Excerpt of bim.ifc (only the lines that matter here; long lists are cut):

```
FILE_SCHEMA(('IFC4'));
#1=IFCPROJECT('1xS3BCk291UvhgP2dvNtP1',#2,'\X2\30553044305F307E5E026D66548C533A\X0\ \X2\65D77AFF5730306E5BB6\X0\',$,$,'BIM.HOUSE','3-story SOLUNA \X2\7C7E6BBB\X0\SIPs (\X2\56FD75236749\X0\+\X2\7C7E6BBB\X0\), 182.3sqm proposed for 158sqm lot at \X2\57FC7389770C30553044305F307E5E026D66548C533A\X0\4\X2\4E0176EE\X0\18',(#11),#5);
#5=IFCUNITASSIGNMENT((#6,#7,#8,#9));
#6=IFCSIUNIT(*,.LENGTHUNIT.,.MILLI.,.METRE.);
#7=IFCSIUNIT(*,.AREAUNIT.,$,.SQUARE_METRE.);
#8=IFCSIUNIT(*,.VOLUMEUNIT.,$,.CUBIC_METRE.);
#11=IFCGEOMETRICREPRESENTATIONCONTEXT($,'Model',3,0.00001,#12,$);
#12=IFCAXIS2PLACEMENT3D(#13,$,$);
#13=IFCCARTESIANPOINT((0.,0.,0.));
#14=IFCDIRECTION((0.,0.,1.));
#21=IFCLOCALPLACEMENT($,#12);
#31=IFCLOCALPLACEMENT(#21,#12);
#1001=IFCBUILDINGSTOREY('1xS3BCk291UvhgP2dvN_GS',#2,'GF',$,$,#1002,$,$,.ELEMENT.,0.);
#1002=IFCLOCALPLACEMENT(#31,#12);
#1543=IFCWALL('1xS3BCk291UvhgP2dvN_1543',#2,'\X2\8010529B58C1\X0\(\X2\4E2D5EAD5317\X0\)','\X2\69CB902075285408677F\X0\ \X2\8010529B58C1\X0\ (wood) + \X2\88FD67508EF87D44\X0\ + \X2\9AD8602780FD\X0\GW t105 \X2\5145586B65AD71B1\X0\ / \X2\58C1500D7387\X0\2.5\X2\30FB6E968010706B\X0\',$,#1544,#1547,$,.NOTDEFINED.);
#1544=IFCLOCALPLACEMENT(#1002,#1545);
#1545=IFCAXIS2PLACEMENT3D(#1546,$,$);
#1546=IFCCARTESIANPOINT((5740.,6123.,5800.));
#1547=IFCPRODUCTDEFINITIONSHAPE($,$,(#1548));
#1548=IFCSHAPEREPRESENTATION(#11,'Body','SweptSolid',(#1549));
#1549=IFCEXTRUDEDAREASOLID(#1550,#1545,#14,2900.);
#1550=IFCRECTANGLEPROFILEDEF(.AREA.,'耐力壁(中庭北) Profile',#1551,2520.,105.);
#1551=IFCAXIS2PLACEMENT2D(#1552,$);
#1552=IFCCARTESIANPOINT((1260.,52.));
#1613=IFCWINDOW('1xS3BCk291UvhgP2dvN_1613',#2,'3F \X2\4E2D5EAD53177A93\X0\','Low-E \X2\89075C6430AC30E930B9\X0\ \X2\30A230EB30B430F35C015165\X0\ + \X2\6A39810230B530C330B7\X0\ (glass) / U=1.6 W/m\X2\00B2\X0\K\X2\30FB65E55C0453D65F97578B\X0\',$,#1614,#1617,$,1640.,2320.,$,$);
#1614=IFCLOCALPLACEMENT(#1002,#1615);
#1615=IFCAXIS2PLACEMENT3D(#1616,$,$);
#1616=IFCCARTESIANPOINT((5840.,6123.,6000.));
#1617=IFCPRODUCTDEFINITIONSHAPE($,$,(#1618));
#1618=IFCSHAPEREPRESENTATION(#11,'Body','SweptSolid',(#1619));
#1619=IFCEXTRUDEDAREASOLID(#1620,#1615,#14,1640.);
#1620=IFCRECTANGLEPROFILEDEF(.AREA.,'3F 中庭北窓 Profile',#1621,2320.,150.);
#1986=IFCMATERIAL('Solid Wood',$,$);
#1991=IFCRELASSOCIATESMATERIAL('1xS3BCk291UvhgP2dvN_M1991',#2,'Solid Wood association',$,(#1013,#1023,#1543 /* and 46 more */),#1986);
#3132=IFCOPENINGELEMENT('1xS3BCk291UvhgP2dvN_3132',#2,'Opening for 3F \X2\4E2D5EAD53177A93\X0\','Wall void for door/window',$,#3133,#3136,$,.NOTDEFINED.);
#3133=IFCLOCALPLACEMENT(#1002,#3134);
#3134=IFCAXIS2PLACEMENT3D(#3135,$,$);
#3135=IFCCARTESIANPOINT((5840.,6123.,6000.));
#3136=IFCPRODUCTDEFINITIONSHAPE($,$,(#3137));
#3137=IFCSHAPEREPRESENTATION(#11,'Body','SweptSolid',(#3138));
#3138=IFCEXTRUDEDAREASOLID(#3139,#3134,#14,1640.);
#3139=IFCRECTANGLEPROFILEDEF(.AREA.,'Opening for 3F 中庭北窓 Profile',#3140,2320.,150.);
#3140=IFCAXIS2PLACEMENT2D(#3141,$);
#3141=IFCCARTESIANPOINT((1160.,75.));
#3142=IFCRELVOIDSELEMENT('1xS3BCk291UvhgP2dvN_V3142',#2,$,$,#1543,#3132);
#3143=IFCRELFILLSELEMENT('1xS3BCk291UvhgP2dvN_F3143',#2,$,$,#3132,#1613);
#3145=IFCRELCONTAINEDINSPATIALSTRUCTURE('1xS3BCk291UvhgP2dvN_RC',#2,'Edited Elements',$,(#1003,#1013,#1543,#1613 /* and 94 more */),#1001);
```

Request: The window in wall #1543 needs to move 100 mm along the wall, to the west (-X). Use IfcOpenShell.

```python
import ifcopenshell
import ifcopenshell.api.geometry
import ifcopenshell.util.placement
import ifcopenshell.util.unit

model = ifcopenshell.open("bim.ifc")
unit_scale = ifcopenshell.util.unit.calculate_unit_scale(model)

window = model.by_id(1613)
opening = window.FillsVoids[0].RelatingOpeningElement
wall = opening.VoidsElements[0].RelatingBuildingElement

wall_matrix = ifcopenshell.util.placement.get_local_placement(wall.ObjectPlacement)
shift = wall_matrix[:3, 0] * -0.1 / unit_scale
before = ifcopenshell.util.placement.get_local_placement(window.ObjectPlacement)[:3, 3].copy()

# The window is not placed relative to its opening, so move both.
for product in (opening, window):
    matrix = ifcopenshell.util.placement.get_local_placement(product.ObjectPlacement)
    matrix[:3, 3] += shift
    ifcopenshell.api.geometry.edit_object_placement(model, product=product, matrix=matrix, is_si=False)

after = ifcopenshell.util.placement.get_local_placement(window.ObjectPlacement)[:3, 3]
print("window moved by", (after - before).round(3) + 0.0)

model.write("bim_v2.ifc")
```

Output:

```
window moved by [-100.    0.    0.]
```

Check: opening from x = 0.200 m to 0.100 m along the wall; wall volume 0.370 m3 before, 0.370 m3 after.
